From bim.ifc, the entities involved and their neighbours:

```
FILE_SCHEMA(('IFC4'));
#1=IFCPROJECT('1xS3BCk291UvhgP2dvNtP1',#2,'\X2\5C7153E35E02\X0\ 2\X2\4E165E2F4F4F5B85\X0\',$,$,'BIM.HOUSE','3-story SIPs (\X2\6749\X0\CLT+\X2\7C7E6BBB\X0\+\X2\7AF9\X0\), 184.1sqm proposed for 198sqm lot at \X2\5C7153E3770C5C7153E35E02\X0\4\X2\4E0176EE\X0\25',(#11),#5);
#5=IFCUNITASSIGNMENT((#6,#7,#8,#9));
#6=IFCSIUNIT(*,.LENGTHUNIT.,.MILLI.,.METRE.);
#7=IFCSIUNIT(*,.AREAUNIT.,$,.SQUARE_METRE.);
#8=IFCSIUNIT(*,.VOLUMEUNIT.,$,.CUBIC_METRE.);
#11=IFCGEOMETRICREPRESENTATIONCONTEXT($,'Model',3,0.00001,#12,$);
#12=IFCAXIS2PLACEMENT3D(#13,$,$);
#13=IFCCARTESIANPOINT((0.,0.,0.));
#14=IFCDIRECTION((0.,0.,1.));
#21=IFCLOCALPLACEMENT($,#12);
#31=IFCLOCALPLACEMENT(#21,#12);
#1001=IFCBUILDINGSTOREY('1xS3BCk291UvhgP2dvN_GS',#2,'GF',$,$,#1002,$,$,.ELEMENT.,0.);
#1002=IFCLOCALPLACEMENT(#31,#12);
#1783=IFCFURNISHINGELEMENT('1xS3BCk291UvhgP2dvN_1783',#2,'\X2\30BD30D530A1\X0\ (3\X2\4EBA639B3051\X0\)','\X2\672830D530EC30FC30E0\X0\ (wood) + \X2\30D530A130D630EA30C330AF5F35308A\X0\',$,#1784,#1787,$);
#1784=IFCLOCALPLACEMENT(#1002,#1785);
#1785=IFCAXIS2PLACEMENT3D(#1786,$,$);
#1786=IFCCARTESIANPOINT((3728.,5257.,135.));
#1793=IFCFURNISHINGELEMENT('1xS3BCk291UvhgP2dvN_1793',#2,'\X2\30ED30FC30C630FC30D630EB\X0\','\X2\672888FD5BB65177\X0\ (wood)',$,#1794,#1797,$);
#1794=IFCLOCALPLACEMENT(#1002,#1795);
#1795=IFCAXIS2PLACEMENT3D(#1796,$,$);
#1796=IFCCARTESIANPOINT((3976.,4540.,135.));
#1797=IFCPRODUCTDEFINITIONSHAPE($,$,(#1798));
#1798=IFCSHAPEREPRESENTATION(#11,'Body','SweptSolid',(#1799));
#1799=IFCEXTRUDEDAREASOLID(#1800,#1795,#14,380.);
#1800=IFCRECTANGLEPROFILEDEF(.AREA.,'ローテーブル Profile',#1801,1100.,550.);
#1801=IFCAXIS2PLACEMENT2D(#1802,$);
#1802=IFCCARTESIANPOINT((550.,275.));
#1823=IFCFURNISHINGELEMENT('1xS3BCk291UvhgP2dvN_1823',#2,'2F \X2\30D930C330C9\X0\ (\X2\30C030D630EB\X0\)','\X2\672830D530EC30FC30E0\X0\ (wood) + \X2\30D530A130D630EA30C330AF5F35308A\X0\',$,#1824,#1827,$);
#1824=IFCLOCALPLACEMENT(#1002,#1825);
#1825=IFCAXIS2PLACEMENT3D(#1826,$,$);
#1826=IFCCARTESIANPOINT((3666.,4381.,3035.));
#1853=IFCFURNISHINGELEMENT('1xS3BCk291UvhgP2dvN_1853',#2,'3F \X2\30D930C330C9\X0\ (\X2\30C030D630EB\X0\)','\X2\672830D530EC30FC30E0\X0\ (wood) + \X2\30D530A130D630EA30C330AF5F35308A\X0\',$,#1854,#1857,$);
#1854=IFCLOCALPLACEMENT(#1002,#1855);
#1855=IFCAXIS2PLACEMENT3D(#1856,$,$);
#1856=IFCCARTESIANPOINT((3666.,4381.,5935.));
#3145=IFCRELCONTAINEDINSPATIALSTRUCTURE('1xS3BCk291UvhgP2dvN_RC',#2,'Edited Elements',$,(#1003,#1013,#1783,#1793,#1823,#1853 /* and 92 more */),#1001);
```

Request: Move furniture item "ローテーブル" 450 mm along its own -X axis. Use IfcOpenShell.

```python
import ifcopenshell
import ifcopenshell.api.geometry
import ifcopenshell.util.placement

model = ifcopenshell.open("bim.ifc")

item = model.by_id(1793)
matrix = ifcopenshell.util.placement.get_local_placement(item.ObjectPlacement)
matrix[:3, 3] -= matrix[:3, 0] * 450.0
ifcopenshell.api.geometry.edit_object_placement(model, product=item, matrix=matrix, is_si=False)

print(ifcopenshell.util.placement.get_local_placement(item.ObjectPlacement).round(3) + 0.0)

model.write("bim_updated.ifc")
```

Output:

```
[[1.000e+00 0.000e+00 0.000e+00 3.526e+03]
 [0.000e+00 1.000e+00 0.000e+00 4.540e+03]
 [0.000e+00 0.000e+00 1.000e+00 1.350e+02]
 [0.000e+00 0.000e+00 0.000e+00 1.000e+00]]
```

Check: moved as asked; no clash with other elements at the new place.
